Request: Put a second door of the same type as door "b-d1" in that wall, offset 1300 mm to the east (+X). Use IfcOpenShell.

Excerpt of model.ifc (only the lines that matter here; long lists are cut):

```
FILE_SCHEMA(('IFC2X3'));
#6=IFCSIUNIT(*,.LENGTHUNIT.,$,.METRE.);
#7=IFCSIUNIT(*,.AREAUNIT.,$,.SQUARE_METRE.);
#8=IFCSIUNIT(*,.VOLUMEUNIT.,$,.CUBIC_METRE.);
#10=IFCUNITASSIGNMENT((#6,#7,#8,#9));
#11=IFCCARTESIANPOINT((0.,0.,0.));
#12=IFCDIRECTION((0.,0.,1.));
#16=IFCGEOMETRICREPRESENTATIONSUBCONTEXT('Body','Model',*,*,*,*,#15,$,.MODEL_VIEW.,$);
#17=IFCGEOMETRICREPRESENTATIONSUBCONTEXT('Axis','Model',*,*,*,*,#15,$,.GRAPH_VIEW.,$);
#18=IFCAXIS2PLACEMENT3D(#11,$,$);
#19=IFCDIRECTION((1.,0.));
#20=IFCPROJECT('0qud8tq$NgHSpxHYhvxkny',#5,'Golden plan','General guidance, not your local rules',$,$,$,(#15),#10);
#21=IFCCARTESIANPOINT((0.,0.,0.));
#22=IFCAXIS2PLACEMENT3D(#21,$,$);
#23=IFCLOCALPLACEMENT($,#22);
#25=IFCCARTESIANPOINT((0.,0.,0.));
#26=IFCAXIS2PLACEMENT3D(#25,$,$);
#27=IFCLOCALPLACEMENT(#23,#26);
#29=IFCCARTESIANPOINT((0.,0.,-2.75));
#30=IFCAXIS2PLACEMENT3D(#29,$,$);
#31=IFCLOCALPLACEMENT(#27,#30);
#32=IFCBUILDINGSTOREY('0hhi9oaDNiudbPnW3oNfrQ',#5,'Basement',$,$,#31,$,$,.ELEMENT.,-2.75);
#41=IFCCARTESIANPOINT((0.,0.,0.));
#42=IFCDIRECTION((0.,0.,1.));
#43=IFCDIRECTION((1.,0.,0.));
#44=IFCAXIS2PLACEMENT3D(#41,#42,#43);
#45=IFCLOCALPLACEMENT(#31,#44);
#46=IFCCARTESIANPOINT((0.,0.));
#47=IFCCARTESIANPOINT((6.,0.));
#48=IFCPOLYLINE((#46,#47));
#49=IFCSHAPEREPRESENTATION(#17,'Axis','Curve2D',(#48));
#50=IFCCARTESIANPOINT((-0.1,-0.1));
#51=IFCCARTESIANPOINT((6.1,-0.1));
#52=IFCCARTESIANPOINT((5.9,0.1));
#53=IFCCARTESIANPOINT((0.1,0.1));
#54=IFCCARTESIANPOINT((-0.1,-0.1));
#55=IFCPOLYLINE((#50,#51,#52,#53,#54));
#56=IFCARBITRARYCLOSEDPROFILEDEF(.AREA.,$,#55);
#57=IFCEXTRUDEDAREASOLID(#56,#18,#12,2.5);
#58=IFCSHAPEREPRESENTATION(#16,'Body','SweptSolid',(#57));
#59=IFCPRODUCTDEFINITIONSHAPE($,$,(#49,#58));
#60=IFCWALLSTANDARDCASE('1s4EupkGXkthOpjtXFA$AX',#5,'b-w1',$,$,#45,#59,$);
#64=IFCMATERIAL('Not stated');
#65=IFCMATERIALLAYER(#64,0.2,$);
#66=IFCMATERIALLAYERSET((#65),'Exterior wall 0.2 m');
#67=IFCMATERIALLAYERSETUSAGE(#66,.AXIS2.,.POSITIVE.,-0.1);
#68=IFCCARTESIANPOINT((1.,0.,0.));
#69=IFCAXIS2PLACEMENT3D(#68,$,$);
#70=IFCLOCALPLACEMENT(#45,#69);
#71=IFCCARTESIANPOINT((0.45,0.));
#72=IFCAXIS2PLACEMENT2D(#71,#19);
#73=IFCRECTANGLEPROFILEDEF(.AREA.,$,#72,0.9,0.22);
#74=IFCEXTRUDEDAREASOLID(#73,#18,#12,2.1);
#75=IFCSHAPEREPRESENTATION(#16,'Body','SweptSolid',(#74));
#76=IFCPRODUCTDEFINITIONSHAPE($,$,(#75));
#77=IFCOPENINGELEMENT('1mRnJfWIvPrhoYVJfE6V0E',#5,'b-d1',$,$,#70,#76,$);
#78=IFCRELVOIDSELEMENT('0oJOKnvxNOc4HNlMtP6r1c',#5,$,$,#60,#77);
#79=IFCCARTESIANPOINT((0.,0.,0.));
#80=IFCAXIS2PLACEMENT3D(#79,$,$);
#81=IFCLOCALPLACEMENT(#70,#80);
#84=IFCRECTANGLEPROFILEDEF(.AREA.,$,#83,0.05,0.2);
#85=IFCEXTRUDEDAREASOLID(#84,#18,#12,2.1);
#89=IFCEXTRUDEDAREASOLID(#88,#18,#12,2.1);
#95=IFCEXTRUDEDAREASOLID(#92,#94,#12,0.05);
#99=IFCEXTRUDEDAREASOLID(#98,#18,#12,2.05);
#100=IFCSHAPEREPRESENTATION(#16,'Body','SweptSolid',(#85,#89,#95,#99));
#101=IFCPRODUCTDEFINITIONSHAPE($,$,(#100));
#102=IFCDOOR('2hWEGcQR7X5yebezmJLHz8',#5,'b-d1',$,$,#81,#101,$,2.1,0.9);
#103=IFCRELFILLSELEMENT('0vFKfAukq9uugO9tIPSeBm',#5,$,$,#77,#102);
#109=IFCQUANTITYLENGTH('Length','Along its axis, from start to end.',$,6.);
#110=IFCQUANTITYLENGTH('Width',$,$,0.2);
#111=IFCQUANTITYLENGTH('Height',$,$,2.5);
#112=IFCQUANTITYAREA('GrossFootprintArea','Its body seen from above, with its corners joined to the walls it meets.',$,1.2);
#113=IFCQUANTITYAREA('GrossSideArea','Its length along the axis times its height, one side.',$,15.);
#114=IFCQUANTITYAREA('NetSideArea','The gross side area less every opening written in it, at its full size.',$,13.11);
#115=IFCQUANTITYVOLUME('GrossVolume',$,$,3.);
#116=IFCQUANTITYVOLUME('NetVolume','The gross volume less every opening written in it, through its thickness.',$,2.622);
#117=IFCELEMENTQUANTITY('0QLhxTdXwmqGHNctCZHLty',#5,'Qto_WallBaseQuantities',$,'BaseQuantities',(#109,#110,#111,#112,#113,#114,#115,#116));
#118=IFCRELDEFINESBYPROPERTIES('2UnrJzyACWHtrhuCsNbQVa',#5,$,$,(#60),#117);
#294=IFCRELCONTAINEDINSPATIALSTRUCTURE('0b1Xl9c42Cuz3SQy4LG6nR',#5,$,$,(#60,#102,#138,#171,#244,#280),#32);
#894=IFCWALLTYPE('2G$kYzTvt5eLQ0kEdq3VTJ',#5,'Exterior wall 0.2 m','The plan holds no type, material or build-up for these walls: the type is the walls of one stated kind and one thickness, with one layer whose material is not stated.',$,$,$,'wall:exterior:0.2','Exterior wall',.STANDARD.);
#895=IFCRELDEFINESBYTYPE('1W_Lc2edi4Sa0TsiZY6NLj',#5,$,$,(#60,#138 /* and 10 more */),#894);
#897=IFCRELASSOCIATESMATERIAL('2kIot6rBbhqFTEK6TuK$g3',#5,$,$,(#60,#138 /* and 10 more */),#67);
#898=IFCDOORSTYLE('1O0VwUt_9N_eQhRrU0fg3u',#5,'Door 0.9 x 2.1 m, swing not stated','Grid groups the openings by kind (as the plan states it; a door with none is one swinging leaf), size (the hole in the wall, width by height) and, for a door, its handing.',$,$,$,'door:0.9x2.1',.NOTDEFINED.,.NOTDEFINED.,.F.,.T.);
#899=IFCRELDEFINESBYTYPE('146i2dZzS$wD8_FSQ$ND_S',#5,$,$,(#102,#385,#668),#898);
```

```python
import ifcopenshell
import ifcopenshell.api.feature
import ifcopenshell.api.geometry
import ifcopenshell.api.pset
import ifcopenshell.api.root
import ifcopenshell.geom
import ifcopenshell.util.element
import ifcopenshell.util.placement
import ifcopenshell.util.shape
import ifcopenshell.util.unit

model = ifcopenshell.open("model.ifc")
unit_scale = ifcopenshell.util.unit.calculate_unit_scale(model)
area_scale = ifcopenshell.util.unit.calculate_unit_scale(model, "AREAUNIT")
volume_scale = ifcopenshell.util.unit.calculate_unit_scale(model, "VOLUMEUNIT")
settings = ifcopenshell.geom.settings()


def volume(element):
    """Net volume in cubic metres, openings subtracted."""
    shape = ifcopenshell.geom.create_shape(settings, element)
    return ifcopenshell.util.shape.get_volume(shape.geometry)


def reuse_history(source, copy):
    """copy_class also copies each property set's owner history, people and application; keep the originals."""
    for rel in copy.IsDefinedBy:
        if rel.is_a("IfcRelDefinesByProperties") and (history := rel.RelatingPropertyDefinition.OwnerHistory):
            rel.RelatingPropertyDefinition.OwnerHistory = source.OwnerHistory
            ifcopenshell.util.element.remove_deep2(model, history)


door = model.by_id(102)
opening = door.FillsVoids[0].RelatingOpeningElement
wall = opening.VoidsElements[0].RelatingBuildingElement
before = volume(wall)
shift = ifcopenshell.util.placement.get_local_placement(wall.ObjectPlacement)[:3, 0] * 1.3 / unit_scale

# copy_class copies the void relationship, type, container and properties, but no geometry.
new_opening = ifcopenshell.api.root.copy_class(model, product=opening)
new_opening.Representation = ifcopenshell.util.element.copy_deep(
    model, opening.Representation, exclude=["IfcGeometricRepresentationContext", "IfcRepresentationMap"]
)
new_door = ifcopenshell.api.root.copy_class(model, product=door)
new_door.Representation = ifcopenshell.util.element.copy_deep(
    model, door.Representation, exclude=["IfcGeometricRepresentationContext", "IfcRepresentationMap"]
)
reuse_history(door, new_door)
fills = ifcopenshell.api.feature.add_filling(model, opening=new_opening, element=new_door)
fills.OwnerHistory = new_door.OwnerHistory  # required in IFC2X3

for old, new in ((opening, new_opening), (door, new_door)):
    matrix = ifcopenshell.util.placement.get_local_placement(old.ObjectPlacement)
    matrix[:3, 3] += shift
    ifcopenshell.api.geometry.edit_object_placement(model, product=new, matrix=matrix, is_si=False)

after = volume(wall)
thickness = 0.2  # wall thickness in metres

# Update the wall's stored quantities.
qto = model.by_id(ifcopenshell.util.element.get_pset(wall, "Qto_WallBaseQuantities", should_inherit=False)["id"])
ifcopenshell.api.pset.edit_qto(model, qto=qto, properties={
    "NetSideArea": after / thickness / area_scale,
    "NetVolume": after / volume_scale,
})

print(f"wall volume {before:.3f} -> {after:.3f} m3")

model.write("model_updated.ifc")
```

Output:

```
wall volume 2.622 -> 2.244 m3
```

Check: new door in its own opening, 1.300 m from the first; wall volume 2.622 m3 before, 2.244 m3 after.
